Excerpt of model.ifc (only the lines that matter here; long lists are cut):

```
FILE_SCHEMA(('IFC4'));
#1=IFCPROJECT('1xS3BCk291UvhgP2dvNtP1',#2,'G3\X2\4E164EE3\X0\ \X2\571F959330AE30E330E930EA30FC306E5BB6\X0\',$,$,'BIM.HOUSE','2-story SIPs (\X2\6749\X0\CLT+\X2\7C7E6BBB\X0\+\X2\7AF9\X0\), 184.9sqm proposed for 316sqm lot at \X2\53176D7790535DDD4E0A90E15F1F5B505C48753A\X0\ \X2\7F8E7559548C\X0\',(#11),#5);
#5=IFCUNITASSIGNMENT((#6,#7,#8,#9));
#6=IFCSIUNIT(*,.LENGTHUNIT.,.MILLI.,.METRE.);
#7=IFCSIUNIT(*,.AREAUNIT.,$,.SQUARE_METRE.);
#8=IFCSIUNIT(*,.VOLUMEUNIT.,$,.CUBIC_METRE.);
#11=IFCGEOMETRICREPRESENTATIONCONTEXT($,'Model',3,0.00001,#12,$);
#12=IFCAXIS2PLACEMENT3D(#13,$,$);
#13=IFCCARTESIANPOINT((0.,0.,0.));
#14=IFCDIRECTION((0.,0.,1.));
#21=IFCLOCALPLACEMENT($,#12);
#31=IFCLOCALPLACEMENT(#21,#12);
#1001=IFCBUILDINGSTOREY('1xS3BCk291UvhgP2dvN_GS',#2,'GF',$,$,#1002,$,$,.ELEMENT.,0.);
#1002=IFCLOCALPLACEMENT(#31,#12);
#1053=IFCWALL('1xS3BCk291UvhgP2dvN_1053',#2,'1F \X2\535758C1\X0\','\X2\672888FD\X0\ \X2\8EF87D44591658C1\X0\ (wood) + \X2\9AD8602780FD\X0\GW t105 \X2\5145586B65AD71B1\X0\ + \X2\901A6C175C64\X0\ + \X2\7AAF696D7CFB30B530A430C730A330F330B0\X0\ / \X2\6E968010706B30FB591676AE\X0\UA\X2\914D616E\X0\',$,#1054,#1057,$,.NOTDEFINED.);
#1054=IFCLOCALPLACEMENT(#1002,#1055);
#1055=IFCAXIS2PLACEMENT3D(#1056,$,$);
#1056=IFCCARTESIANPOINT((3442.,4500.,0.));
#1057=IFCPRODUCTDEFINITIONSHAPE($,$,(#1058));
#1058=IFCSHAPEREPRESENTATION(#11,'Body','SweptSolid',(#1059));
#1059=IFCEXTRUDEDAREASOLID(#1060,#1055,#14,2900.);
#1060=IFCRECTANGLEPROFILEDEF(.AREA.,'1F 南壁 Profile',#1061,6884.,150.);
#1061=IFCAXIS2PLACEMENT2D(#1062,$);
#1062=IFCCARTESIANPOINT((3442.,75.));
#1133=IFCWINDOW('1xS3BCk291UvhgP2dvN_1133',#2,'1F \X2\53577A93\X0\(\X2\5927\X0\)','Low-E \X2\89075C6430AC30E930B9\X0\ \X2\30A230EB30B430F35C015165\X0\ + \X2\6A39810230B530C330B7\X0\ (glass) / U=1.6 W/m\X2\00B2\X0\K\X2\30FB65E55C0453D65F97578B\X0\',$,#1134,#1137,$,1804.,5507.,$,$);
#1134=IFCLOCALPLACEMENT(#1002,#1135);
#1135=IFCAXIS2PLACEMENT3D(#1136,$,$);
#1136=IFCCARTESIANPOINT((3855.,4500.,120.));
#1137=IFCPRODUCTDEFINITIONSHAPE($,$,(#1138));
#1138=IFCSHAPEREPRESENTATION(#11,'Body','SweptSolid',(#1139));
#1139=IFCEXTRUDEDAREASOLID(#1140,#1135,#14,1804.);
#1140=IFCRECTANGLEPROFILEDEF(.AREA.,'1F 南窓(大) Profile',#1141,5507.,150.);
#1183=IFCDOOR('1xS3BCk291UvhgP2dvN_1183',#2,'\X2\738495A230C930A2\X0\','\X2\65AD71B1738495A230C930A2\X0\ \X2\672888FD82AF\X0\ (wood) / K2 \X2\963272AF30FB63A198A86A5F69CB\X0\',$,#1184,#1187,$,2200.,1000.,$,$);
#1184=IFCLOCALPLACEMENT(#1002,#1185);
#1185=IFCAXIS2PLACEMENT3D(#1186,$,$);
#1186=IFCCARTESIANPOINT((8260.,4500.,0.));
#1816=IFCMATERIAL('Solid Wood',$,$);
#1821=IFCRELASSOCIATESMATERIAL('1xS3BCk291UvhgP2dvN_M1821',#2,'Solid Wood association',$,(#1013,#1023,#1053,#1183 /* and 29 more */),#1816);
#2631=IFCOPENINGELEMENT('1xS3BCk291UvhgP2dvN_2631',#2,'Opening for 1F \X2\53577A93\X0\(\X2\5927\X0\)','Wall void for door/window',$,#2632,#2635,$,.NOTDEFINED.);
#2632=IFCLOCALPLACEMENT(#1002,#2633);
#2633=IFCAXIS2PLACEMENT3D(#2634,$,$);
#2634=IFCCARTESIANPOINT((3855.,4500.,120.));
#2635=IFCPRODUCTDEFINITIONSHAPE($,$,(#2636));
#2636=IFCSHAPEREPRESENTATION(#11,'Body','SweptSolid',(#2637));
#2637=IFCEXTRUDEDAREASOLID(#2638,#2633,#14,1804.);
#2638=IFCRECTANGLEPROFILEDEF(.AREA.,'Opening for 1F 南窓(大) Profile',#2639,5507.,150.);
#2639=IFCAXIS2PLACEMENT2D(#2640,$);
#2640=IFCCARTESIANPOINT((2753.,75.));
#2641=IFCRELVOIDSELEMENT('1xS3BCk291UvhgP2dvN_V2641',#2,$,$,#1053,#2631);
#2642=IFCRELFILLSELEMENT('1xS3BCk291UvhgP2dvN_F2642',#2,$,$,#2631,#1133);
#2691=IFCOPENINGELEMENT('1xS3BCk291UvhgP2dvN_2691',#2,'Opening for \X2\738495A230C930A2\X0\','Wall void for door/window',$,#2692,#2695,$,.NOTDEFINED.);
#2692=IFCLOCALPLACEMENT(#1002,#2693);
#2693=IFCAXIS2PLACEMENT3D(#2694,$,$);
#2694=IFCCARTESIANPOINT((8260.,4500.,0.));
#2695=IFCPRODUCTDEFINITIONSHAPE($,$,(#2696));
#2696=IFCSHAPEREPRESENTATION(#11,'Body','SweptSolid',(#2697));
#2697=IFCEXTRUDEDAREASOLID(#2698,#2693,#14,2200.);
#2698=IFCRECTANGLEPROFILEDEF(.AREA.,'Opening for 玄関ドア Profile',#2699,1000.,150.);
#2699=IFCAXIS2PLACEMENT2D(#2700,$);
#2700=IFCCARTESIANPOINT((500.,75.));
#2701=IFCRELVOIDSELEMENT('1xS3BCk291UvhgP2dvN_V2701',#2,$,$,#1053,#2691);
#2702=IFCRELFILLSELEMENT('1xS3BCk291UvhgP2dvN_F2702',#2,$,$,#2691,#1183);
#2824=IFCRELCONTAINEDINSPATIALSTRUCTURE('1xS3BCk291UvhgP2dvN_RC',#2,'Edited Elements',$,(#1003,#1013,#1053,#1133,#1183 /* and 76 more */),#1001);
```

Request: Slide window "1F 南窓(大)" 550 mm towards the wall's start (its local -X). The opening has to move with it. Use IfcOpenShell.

```python
import ifcopenshell
import ifcopenshell.api.geometry
import ifcopenshell.util.placement
import ifcopenshell.util.unit

model = ifcopenshell.open("model.ifc")
unit_scale = ifcopenshell.util.unit.calculate_unit_scale(model)

window = model.by_guid("1xS3BCk291UvhgP2dvN_1133")
opening = window.FillsVoids[0].RelatingOpeningElement
wall = opening.VoidsElements[0].RelatingBuildingElement

wall_matrix = ifcopenshell.util.placement.get_local_placement(wall.ObjectPlacement)
shift = wall_matrix[:3, 0] * -0.55 / unit_scale
before = ifcopenshell.util.placement.get_local_placement(window.ObjectPlacement)[:3, 3].copy()

# The window is not placed relative to its opening, so move both.
for product in (opening, window):
    matrix = ifcopenshell.util.placement.get_local_placement(product.ObjectPlacement)
    matrix[:3, 3] += shift
    ifcopenshell.api.geometry.edit_object_placement(model, product=product, matrix=matrix, is_si=False)

after = ifcopenshell.util.placement.get_local_placement(window.ObjectPlacement)[:3, 3]
print("window moved by", (after - before).round(3) + 0.0)

model.write("model_edited.ifc")
```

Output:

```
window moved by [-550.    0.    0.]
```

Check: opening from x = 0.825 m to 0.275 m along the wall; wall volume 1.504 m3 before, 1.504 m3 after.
